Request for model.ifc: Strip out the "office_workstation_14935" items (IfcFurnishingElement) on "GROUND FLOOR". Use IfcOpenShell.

First a look at what the model holds.

```python
import ifcopenshell
import ifcopenshell.util.element

model = ifcopenshell.open("model.ifc")
print(model.schema)
storey = next(s for s in model.by_type("IfcBuildingStorey") if s.Name == "GROUND FLOOR")
furniture = [e for e in ifcopenshell.util.element.get_decomposition(storey) if e.is_a("IfcFurnishingElement")]
seen = {}
for e in furniture:
    element_type = ifcopenshell.util.element.get_type(e)
    name = element_type.Name if element_type not in (None, e) else None
    seen[name] = seen.get(name, 0) + 1
for name, count in sorted(seen.items(), key=str):
    print(count, "x", name)
```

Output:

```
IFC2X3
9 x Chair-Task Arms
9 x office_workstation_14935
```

```python
import ifcopenshell
import ifcopenshell.api.root
import ifcopenshell.util.element

model = ifcopenshell.open("model.ifc")

storey = next(s for s in model.by_type("IfcBuildingStorey") if s.Name == "GROUND FLOOR")
furniture = [e for e in ifcopenshell.util.element.get_decomposition(storey) if e.is_a("IfcFurnishingElement")]
targets = [e for e in furniture if (t := ifcopenshell.util.element.get_type(e)) not in (None, e) and t.Name == "office_workstation_14935"]

for e in targets:
    ifcopenshell.api.root.remove_product(model, product=e)
print(len(targets), "removed")

model.write("model_updated.ifc")
```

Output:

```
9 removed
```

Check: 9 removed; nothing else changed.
